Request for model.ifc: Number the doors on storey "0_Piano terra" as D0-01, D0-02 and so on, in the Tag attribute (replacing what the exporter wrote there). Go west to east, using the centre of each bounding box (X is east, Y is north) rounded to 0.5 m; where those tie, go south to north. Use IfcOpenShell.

First a look at what the model holds.

```python
import ifcopenshell
import ifcopenshell.util.element
import ifcopenshell.util.placement

model = ifcopenshell.open("model.ifc")
print(model.schema)
storey = next(s for s in model.by_type("IfcBuildingStorey") if s.Name == "0_Piano terra")
doors = [e for e in ifcopenshell.util.element.get_decomposition(storey) if e.is_a("IfcDoor")]
for e in sorted(doors, key=lambda e: e.id()):
    origin = ifcopenshell.util.placement.get_local_placement(e.ObjectPlacement)[:3, 3]
    print(e.id(), e.Tag, e.Name, origin.round(2) + 0.0, sep=" | ")
```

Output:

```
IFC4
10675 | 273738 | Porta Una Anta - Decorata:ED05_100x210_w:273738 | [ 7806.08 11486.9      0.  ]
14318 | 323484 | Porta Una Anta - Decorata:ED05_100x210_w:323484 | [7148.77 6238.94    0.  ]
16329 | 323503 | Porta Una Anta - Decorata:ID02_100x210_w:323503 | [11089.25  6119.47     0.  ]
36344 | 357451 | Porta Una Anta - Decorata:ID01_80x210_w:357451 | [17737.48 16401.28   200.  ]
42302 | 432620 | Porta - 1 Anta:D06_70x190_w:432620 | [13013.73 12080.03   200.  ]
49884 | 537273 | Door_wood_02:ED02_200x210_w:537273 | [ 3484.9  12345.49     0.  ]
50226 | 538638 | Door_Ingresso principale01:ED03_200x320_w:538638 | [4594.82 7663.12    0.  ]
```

```python
import ifcopenshell
import ifcopenshell.geom
import ifcopenshell.util.element
import ifcopenshell.util.shape

model = ifcopenshell.open("model.ifc")
settings = ifcopenshell.geom.settings()
settings.set("use-world-coords", True)


def centre(element):
    shape = ifcopenshell.geom.create_shape(settings, element)
    return ifcopenshell.util.shape.get_bbox_centroid(shape.geometry)


storey = next(s for s in model.by_type("IfcBuildingStorey") if s.Name == "0_Piano terra")
doors = [e for e in ifcopenshell.util.element.get_decomposition(storey) if e.is_a("IfcDoor")]

# Insertion points can sit at a corner or the storey origin, so sort by the geometry (in metres).
centres = {e: centre(e) for e in doors}
doors.sort(key=lambda e: (round(centres[e][0] / 0.5), centres[e][1]))

for i, e in enumerate(doors, start=1):
    number = f"D0-{i:02d}"
    e.Tag = number
    print(e.id(), number)

model.write("model_rev.ifc")
```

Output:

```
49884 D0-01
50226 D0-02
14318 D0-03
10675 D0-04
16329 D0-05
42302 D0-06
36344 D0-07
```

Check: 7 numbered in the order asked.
